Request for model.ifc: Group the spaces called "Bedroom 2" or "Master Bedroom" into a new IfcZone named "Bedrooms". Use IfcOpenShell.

First a look at what the model holds.

```python
import ifcopenshell

model = ifcopenshell.open("model.ifc")
print(model.schema)
seen = {}
for space in model.by_type("IfcSpace"):
    seen[space.LongName] = seen.get(space.LongName, 0) + 1
for name, count in sorted(seen.items(), key=str):
    print(count, "x", name)
print("zones:", [z.Name for z in model.by_type("IfcZone")][:20])
```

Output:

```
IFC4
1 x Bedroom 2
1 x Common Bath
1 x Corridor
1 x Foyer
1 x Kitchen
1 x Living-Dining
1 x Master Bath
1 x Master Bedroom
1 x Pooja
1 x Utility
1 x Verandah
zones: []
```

```python
import ifcopenshell
import ifcopenshell.api.group
import ifcopenshell.api.root

model = ifcopenshell.open("model.ifc")

names = {"Bedroom 2", "Master Bedroom"}
spaces = [s for s in model.by_type("IfcSpace") if s.LongName in names]

zone = ifcopenshell.api.root.create_entity(model, ifc_class="IfcZone", name="Bedrooms")
ifcopenshell.api.group.assign_group(model, products=spaces, group=zone)
print(len(spaces), "spaces in", zone.Name)

model.write("model_updated.ifc")
```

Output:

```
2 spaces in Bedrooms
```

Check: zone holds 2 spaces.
